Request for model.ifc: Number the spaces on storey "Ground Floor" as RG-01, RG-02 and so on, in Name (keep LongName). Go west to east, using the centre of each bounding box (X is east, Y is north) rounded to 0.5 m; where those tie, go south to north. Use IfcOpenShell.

First a look at what the model holds.

```python
import ifcopenshell
import ifcopenshell.util.element
import ifcopenshell.util.placement

model = ifcopenshell.open("model.ifc")
print(model.schema)
storey = next(s for s in model.by_type("IfcBuildingStorey") if s.Name == "Ground Floor")
spaces = [e for e in ifcopenshell.util.element.get_decomposition(storey) if e.is_a("IfcSpace")]
for e in sorted(spaces, key=lambda e: e.id()):
    origin = ifcopenshell.util.placement.get_local_placement(e.ObjectPlacement)[:3, 3]
    print(e.id(), e.Name, e.LongName, origin.round(2) + 0.0, sep=" | ")
```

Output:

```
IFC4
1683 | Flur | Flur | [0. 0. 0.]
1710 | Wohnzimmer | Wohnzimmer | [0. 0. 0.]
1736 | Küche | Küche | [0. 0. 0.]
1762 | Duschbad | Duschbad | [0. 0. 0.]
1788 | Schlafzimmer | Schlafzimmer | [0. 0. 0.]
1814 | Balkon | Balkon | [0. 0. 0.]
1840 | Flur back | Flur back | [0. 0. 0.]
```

```python
import ifcopenshell
import ifcopenshell.geom
import ifcopenshell.util.element
import ifcopenshell.util.shape

model = ifcopenshell.open("model.ifc")
settings = ifcopenshell.geom.settings()
settings.set("use-world-coords", True)


def centre(element):
    shape = ifcopenshell.geom.create_shape(settings, element)
    return ifcopenshell.util.shape.get_bbox_centroid(shape.geometry)


storey = next(s for s in model.by_type("IfcBuildingStorey") if s.Name == "Ground Floor")
spaces = [e for e in ifcopenshell.util.element.get_decomposition(storey) if e.is_a("IfcSpace")]

# Insertion points can sit at a corner or the storey origin, so sort by the geometry (in metres).
centres = {e: centre(e) for e in spaces}
spaces.sort(key=lambda e: (round(centres[e][0] / 0.5), centres[e][1]))

for i, e in enumerate(spaces, start=1):
    number = f"RG-{i:02d}"
    e.Name = number
    print(e.id(), number)

model.write("model_v2.ifc")
```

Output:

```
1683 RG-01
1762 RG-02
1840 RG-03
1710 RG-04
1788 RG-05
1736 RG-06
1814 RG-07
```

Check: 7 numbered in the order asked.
